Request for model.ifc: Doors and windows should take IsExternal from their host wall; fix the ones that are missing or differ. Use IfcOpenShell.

First a look at what the model holds.

```python
import ifcopenshell
import ifcopenshell.util.element

model = ifcopenshell.open("model.ifc")
print(model.schema)
seen = {}
for e in model.by_type("IfcDoor") + model.by_type("IfcWindow"):
    if not e.FillsVoids:
        continue
    host = e.FillsVoids[0].RelatingOpeningElement.VoidsElements[0].RelatingBuildingElement
    own = ifcopenshell.util.element.get_pset(e, f"Pset_{e.is_a()[3:].removesuffix('StandardCase')}Common", "IsExternal")
    wall = ifcopenshell.util.element.get_pset(host, "Pset_WallCommon", "IsExternal")
    seen[e.is_a(), own, wall] = seen.get((e.is_a(), own, wall), 0) + 1
for (cls, own, wall), count in sorted(seen.items(), key=str):
    print(count, cls, "IsExternal:", own, "| host wall:", wall)
```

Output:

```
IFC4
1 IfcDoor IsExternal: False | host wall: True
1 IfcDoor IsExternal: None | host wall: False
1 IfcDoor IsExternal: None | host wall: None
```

```python
import ifcopenshell
import ifcopenshell.api.pset
import ifcopenshell.util.element

model = ifcopenshell.open("model.ifc")

count = 0
for ifc_class, pset_name in (("IfcDoor", "Pset_DoorCommon"), ("IfcWindow", "Pset_WindowCommon")):
    for e in model.by_type(ifc_class):
        if not e.FillsVoids:
            continue
        host = e.FillsVoids[0].RelatingOpeningElement.VoidsElements[0].RelatingBuildingElement
        external = ifcopenshell.util.element.get_pset(host, "Pset_WallCommon", "IsExternal")
        if external is None or ifcopenshell.util.element.get_pset(e, pset_name, "IsExternal") == external:
            continue
        pset = ifcopenshell.api.pset.add_pset(model, product=e, name=pset_name)
        ifcopenshell.api.pset.edit_pset(model, pset=pset, properties={"IsExternal": external})
        count += 1

print(count, "updated")

model.write("model-out.ifc")
```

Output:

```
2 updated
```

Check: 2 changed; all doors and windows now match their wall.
